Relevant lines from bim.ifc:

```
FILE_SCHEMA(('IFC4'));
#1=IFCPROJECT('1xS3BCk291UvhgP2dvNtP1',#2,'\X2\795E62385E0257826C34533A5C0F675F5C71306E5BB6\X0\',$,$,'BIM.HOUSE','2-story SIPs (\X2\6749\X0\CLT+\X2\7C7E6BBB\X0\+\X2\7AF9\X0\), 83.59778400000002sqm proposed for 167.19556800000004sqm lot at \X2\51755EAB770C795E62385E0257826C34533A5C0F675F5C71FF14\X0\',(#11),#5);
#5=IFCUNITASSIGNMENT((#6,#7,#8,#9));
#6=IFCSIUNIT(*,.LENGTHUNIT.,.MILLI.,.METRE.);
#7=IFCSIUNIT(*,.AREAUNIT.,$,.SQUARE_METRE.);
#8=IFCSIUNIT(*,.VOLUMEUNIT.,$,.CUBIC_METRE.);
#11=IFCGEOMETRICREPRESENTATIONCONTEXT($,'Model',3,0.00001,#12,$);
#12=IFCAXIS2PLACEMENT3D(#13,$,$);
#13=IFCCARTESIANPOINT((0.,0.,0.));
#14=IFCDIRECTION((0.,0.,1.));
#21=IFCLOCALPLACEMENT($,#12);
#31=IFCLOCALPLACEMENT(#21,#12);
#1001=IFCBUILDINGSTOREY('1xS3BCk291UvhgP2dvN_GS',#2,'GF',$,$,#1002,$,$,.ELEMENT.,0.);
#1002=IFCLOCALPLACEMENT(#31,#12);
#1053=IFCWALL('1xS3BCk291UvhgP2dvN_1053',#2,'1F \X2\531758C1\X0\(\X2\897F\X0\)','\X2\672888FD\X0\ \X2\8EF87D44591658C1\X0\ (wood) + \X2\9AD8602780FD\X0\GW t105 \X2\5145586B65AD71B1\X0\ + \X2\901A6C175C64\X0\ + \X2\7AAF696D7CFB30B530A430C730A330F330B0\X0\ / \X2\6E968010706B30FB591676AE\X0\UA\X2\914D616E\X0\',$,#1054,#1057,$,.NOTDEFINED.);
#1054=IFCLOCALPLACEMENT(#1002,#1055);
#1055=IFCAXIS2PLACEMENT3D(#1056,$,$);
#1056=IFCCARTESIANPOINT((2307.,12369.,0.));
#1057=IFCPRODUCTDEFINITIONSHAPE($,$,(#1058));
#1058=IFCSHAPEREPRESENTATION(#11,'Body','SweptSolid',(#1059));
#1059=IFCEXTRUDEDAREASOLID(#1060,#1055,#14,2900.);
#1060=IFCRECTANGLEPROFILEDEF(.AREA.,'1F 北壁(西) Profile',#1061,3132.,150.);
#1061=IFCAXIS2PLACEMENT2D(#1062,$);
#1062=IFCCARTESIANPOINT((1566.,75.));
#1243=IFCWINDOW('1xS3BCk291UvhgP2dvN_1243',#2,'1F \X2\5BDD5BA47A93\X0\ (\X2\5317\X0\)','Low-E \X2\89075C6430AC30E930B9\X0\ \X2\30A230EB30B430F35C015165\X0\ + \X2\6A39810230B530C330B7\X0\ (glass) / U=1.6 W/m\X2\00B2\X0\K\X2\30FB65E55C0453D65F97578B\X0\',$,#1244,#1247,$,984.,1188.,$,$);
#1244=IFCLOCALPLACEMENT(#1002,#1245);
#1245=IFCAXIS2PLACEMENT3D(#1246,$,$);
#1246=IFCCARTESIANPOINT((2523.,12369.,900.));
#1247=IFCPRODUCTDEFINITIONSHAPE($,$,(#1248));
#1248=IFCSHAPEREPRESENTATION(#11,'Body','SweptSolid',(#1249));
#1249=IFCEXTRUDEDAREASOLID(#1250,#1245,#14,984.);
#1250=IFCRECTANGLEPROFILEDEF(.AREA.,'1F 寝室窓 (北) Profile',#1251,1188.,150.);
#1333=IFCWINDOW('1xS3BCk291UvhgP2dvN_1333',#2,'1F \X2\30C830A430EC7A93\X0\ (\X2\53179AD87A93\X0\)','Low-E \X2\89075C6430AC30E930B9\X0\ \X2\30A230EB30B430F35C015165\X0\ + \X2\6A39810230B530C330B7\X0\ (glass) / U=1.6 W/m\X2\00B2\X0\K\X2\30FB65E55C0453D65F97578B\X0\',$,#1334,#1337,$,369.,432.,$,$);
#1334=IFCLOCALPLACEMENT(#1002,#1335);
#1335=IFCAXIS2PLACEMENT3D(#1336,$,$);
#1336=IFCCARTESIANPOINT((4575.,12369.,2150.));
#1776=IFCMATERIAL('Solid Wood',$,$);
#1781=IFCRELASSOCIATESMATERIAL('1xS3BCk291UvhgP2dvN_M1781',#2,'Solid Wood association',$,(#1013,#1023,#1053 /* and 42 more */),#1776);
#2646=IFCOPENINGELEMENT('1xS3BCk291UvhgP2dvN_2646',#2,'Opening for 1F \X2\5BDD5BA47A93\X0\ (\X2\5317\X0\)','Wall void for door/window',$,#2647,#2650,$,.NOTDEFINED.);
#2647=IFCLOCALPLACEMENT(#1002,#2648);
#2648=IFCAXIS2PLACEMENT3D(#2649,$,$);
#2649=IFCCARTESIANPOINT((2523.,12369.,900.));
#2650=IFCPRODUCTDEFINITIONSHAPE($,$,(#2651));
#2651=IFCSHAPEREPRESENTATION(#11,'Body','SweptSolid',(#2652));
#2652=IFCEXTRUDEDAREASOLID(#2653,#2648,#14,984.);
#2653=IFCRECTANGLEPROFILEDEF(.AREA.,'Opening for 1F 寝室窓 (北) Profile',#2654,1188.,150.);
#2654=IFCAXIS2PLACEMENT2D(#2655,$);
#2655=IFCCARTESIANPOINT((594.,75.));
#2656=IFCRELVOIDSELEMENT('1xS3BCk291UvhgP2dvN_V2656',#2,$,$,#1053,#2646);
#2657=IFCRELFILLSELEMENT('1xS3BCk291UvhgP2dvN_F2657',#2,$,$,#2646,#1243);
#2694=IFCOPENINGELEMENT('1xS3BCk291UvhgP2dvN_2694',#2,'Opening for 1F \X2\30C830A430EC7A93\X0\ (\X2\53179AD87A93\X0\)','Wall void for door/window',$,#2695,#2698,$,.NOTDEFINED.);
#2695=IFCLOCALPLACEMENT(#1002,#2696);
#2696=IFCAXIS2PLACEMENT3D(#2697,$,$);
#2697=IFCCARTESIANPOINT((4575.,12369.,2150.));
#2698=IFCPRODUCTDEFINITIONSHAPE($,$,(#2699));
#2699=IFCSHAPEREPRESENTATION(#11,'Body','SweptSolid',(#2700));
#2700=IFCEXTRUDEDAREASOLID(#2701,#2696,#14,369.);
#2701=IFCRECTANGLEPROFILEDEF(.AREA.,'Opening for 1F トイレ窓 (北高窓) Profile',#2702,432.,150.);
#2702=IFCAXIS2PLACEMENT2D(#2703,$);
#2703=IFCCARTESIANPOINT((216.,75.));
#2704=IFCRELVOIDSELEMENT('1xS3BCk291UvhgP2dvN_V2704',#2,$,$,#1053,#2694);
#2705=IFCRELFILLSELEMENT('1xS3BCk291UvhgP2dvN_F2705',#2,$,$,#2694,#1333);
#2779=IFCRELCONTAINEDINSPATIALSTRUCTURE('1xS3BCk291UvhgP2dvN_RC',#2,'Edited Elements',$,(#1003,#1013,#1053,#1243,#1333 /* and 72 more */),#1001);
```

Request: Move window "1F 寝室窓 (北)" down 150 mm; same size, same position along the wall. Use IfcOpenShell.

```python
import numpy as np
import ifcopenshell
import ifcopenshell.api.geometry
import ifcopenshell.util.placement
import ifcopenshell.util.unit

model = ifcopenshell.open("bim.ifc")
unit_scale = ifcopenshell.util.unit.calculate_unit_scale(model)

window = model.by_id(1243)
opening = window.FillsVoids[0].RelatingOpeningElement
dz = -0.15 / unit_scale

shift = np.array([0.0, 0.0, dz])
# The window is not placed relative to its opening, so move both.
for product in (opening, window):
    matrix = ifcopenshell.util.placement.get_local_placement(product.ObjectPlacement)
    matrix[:3, 3] += shift
    ifcopenshell.api.geometry.edit_object_placement(model, product=product, matrix=matrix, is_si=False)

print(f"moved by {dz * unit_scale:+.3f} m")

model.write("bim_rev.ifc")
```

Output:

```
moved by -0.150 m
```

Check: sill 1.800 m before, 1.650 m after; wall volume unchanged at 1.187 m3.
